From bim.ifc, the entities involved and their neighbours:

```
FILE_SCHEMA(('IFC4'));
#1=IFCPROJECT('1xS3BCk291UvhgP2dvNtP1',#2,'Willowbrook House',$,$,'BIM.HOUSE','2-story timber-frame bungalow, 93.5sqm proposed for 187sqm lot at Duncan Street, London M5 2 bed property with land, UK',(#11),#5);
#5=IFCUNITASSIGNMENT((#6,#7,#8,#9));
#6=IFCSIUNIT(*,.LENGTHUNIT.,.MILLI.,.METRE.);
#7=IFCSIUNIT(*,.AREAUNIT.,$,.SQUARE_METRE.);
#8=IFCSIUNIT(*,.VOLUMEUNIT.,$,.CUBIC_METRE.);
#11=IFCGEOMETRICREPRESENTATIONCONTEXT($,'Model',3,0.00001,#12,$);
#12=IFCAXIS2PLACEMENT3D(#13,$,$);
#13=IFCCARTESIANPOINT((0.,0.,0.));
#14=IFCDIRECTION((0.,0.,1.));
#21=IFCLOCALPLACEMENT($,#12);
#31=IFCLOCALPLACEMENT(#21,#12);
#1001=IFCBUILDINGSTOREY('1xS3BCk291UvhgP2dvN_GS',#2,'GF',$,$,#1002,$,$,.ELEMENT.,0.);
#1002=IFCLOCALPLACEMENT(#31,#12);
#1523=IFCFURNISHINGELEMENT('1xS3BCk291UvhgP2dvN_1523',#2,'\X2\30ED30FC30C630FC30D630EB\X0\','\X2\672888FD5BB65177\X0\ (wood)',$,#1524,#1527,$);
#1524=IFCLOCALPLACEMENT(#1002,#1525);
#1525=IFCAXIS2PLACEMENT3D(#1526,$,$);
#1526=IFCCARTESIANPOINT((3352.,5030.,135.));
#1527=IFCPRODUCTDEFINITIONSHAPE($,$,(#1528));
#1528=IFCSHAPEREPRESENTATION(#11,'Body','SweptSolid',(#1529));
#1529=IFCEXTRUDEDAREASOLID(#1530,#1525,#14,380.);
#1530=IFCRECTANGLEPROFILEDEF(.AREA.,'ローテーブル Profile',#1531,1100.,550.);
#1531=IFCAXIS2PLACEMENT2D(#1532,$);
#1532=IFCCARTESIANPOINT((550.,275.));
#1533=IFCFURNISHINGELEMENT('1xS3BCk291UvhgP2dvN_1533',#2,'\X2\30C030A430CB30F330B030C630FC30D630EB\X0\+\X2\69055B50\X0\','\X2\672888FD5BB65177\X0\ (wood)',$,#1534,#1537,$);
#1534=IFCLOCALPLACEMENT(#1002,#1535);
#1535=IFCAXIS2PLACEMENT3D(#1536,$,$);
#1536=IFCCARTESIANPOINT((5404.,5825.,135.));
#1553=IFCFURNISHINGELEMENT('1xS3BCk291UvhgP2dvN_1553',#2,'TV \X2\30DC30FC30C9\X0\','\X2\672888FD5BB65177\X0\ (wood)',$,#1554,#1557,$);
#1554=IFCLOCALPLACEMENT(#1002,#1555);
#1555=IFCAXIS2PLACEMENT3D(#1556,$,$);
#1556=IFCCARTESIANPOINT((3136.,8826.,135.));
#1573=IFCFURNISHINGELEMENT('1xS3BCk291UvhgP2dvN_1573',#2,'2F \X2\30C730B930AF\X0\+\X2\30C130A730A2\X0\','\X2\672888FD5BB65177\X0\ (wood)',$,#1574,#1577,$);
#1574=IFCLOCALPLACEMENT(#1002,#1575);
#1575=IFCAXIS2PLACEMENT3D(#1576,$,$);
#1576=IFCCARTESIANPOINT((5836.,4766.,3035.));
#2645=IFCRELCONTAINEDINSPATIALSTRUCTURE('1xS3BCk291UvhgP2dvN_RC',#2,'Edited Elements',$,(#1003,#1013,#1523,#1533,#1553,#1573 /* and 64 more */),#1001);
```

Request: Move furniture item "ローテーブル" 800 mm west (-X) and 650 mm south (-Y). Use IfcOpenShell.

```python
import ifcopenshell
import ifcopenshell.api.geometry
import ifcopenshell.util.placement
import ifcopenshell.util.unit

model = ifcopenshell.open("bim.ifc")
unit_scale = ifcopenshell.util.unit.calculate_unit_scale(model)

item = model.by_guid("1xS3BCk291UvhgP2dvN_1523")
matrix = ifcopenshell.util.placement.get_local_placement(item.ObjectPlacement)
matrix[0, 3] -= 0.8 / unit_scale
matrix[1, 3] -= 0.65 / unit_scale
ifcopenshell.api.geometry.edit_object_placement(model, product=item, matrix=matrix, is_si=False)

print(ifcopenshell.util.placement.get_local_placement(item.ObjectPlacement).round(3) + 0.0)

model.write("bim_updated.ifc")
```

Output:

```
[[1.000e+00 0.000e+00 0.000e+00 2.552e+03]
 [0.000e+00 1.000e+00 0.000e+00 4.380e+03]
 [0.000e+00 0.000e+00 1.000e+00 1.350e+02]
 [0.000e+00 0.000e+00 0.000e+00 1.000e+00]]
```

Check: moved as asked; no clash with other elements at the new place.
